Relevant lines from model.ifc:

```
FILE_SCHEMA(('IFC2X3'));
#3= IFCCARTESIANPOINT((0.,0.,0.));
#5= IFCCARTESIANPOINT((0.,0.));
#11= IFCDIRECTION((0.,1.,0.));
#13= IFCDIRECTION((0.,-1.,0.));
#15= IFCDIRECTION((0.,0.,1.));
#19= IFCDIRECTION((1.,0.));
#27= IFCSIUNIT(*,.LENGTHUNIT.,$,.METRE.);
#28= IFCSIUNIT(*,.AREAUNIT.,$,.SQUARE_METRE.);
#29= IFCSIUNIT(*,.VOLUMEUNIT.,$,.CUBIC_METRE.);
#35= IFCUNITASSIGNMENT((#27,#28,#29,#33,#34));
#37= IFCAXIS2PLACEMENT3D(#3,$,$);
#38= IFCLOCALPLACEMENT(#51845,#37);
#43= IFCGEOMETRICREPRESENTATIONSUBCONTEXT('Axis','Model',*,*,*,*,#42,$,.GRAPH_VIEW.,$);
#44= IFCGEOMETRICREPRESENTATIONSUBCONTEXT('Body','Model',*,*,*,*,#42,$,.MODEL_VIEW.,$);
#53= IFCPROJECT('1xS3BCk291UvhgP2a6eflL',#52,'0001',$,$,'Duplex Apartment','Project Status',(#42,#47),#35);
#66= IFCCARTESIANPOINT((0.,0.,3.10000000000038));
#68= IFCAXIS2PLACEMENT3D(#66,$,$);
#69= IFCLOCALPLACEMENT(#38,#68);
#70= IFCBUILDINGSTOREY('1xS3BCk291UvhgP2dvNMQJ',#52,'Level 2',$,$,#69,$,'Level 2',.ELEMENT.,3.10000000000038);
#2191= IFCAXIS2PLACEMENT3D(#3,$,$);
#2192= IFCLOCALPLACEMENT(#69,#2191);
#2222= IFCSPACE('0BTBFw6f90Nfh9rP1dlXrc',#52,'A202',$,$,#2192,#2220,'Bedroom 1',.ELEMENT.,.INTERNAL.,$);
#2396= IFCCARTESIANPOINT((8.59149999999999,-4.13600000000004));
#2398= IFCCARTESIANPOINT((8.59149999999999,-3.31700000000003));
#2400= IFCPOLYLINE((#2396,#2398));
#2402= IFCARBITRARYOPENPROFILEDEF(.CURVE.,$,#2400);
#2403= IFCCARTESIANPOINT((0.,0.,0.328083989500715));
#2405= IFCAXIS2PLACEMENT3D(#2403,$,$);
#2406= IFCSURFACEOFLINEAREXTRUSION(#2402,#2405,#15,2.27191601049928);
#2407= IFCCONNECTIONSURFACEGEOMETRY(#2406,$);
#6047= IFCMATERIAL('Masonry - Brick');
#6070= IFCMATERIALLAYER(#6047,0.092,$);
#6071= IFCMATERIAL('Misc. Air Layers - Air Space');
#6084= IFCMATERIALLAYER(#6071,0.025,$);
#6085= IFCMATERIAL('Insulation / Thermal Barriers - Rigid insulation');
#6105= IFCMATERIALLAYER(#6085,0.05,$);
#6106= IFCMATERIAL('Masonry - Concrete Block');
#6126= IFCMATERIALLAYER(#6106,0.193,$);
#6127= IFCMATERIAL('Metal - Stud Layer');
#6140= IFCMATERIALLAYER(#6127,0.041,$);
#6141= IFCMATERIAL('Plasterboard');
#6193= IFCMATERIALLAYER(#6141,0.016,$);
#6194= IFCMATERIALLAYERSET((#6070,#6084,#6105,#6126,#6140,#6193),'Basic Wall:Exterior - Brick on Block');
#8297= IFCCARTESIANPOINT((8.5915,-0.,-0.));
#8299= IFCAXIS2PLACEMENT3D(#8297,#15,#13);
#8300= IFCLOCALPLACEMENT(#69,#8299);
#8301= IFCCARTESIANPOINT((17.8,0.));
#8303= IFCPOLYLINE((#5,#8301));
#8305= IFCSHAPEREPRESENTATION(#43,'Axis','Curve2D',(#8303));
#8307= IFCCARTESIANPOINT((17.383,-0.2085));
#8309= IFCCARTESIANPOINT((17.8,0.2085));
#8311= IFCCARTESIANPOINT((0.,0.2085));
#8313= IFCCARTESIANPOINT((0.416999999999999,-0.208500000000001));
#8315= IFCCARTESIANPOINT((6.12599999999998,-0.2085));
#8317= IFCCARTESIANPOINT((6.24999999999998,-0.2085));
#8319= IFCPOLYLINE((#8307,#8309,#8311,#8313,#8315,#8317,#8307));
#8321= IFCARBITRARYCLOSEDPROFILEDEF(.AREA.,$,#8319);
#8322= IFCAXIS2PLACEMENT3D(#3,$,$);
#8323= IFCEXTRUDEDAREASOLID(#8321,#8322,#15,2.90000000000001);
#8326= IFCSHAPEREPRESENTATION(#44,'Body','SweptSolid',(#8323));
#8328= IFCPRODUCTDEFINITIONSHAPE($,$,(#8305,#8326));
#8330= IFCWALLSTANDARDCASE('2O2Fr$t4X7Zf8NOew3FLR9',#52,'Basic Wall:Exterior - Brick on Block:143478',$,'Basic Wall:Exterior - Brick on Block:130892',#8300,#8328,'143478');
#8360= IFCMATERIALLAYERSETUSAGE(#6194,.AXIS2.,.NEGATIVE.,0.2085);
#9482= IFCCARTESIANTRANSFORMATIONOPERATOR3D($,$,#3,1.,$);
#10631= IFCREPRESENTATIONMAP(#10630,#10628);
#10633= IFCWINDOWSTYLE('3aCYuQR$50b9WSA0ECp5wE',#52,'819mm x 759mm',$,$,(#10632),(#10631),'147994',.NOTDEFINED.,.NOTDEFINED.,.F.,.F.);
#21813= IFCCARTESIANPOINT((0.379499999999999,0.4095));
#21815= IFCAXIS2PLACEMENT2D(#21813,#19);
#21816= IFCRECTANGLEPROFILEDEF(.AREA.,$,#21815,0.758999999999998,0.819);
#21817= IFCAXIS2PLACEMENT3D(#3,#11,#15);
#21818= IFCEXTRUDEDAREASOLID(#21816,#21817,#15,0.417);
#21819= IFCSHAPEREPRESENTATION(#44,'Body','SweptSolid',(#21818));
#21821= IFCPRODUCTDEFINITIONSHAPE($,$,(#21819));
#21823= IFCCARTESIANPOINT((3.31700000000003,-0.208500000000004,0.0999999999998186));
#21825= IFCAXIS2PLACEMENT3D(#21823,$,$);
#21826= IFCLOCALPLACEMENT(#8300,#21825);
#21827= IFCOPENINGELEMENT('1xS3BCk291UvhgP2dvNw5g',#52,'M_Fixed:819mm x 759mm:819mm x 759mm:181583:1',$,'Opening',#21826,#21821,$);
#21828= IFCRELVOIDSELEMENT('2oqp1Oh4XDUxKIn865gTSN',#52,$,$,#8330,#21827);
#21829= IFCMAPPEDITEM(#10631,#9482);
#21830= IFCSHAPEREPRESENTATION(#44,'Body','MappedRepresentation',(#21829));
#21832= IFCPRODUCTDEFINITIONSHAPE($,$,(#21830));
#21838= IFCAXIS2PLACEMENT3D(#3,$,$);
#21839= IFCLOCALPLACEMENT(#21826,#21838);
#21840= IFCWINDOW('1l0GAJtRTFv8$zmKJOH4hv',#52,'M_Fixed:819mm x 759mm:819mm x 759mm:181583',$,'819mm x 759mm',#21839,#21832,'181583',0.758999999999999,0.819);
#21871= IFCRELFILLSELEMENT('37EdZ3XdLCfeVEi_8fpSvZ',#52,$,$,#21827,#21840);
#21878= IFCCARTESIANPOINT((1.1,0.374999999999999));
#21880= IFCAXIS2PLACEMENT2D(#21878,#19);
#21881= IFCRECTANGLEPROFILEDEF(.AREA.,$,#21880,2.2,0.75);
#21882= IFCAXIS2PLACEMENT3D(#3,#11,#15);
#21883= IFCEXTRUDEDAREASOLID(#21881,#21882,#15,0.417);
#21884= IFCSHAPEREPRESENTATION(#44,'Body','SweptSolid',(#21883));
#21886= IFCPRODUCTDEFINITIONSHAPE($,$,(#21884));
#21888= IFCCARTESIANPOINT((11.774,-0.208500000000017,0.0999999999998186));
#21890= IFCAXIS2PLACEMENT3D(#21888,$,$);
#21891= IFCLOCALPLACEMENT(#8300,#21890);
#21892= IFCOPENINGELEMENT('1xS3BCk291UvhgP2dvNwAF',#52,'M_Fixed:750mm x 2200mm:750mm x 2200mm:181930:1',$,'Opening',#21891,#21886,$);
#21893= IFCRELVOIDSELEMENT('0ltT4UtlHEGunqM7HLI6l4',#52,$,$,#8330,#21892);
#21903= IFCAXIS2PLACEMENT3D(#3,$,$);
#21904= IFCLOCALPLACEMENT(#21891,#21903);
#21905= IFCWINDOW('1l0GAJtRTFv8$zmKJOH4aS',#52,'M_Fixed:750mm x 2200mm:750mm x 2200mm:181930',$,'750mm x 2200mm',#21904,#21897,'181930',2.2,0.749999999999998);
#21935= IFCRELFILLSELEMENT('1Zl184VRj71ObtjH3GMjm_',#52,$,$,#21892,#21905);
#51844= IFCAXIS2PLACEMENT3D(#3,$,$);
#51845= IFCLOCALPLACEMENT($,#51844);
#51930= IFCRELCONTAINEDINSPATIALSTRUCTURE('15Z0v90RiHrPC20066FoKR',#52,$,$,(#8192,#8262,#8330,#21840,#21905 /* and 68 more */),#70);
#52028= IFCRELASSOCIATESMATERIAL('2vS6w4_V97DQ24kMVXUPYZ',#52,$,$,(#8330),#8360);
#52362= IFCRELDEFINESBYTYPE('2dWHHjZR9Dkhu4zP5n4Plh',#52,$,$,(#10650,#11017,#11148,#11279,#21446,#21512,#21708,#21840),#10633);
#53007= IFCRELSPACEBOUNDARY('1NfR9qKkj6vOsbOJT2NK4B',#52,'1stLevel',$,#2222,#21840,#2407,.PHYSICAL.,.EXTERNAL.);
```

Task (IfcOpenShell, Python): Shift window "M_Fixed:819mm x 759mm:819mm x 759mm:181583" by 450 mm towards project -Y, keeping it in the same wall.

```python
import numpy as np
import ifcopenshell
import ifcopenshell.api.geometry
import ifcopenshell.util.placement
import ifcopenshell.util.unit

model = ifcopenshell.open("model.ifc")
unit_scale = ifcopenshell.util.unit.calculate_unit_scale(model)

window = model.by_guid("1l0GAJtRTFv8$zmKJOH4hv")
opening = window.FillsVoids[0].RelatingOpeningElement
wall = opening.VoidsElements[0].RelatingBuildingElement

wall_matrix = ifcopenshell.util.placement.get_local_placement(wall.ObjectPlacement)
shift = wall_matrix[:3, 0] * 0.45 / unit_scale
before = ifcopenshell.util.placement.get_local_placement(window.ObjectPlacement)[:3, 3].copy()

# The window is placed relative to its opening, so it follows when the opening moves.
matrix = ifcopenshell.util.placement.get_local_placement(opening.ObjectPlacement)
matrix[:3, 3] += shift
ifcopenshell.api.geometry.edit_object_placement(
    model, product=opening, matrix=matrix, is_si=False, should_transform_children=True
)

# Space boundary surfaces are stored in each space's coordinates; move them too.
for rel in window.ProvidesBoundaries:
    if not rel.ConnectionGeometry:
        continue
    surface = rel.ConnectionGeometry.SurfaceOnRelatingElement
    space_matrix = ifcopenshell.util.placement.get_local_placement(rel.RelatingSpace.ObjectPlacement)
    point = np.array(surface.Position.Location.Coordinates) + space_matrix[:3, :3].T @ shift
    surface.Position = model.createIfcAxis2Placement3D(
        model.createIfcCartesianPoint(point.tolist()), surface.Position.Axis, surface.Position.RefDirection
    )

after = ifcopenshell.util.placement.get_local_placement(window.ObjectPlacement)[:3, 3]
print("window moved by", (after - before).round(3) + 0.0)

model.write("model_edited.ifc")
```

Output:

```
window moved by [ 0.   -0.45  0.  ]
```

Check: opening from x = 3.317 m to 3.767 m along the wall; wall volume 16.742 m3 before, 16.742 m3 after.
